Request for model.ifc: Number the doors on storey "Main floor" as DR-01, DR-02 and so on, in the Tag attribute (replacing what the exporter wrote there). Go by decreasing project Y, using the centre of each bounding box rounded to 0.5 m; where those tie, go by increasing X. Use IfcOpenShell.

First a look at what the model holds.

```python
import ifcopenshell
import ifcopenshell.util.element
import ifcopenshell.util.placement

model = ifcopenshell.open("model.ifc")
print(model.schema)
storey = next(s for s in model.by_type("IfcBuildingStorey") if s.Name == "Main floor")
doors = [e for e in ifcopenshell.util.element.get_decomposition(storey) if e.is_a("IfcDoor")]
for e in sorted(doors, key=lambda e: e.id()):
    origin = ifcopenshell.util.placement.get_local_placement(e.ObjectPlacement)[:3, 3]
    print(e.id(), e.Tag, e.Name, origin.round(2) + 0.0, sep=" | ")
```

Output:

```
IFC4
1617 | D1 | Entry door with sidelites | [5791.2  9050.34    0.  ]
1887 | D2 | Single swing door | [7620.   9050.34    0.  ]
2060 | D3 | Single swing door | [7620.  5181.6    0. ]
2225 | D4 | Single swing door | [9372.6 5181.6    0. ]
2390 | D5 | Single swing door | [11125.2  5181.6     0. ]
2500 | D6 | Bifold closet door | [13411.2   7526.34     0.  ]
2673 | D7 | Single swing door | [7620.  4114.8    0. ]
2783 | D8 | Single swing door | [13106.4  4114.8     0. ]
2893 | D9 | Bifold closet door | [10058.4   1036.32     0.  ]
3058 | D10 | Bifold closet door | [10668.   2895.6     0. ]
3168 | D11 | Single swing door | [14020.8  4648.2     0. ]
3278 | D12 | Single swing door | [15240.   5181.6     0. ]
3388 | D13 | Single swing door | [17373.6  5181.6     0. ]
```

```python
import ifcopenshell
import ifcopenshell.geom
import ifcopenshell.util.element
import ifcopenshell.util.shape

model = ifcopenshell.open("model.ifc")
settings = ifcopenshell.geom.settings()
settings.set("use-world-coords", True)


def centre(element):
    shape = ifcopenshell.geom.create_shape(settings, element)
    return ifcopenshell.util.shape.get_bbox_centroid(shape.geometry)


storey = next(s for s in model.by_type("IfcBuildingStorey") if s.Name == "Main floor")
doors = [e for e in ifcopenshell.util.element.get_decomposition(storey) if e.is_a("IfcDoor")]

# Insertion points can sit at a corner or the storey origin, so sort by the geometry (in metres).
centres = {e: centre(e) for e in doors}
doors.sort(key=lambda e: (-round(centres[e][1] / 0.5), centres[e][0]))

for i, e in enumerate(doors, start=1):
    number = f"DR-{i:02d}"
    e.Tag = number
    print(e.id(), number)

model.write("model_edited.ifc")
```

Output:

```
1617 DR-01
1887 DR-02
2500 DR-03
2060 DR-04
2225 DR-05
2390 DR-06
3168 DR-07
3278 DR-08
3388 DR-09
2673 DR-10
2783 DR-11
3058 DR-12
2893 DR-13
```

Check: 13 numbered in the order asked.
